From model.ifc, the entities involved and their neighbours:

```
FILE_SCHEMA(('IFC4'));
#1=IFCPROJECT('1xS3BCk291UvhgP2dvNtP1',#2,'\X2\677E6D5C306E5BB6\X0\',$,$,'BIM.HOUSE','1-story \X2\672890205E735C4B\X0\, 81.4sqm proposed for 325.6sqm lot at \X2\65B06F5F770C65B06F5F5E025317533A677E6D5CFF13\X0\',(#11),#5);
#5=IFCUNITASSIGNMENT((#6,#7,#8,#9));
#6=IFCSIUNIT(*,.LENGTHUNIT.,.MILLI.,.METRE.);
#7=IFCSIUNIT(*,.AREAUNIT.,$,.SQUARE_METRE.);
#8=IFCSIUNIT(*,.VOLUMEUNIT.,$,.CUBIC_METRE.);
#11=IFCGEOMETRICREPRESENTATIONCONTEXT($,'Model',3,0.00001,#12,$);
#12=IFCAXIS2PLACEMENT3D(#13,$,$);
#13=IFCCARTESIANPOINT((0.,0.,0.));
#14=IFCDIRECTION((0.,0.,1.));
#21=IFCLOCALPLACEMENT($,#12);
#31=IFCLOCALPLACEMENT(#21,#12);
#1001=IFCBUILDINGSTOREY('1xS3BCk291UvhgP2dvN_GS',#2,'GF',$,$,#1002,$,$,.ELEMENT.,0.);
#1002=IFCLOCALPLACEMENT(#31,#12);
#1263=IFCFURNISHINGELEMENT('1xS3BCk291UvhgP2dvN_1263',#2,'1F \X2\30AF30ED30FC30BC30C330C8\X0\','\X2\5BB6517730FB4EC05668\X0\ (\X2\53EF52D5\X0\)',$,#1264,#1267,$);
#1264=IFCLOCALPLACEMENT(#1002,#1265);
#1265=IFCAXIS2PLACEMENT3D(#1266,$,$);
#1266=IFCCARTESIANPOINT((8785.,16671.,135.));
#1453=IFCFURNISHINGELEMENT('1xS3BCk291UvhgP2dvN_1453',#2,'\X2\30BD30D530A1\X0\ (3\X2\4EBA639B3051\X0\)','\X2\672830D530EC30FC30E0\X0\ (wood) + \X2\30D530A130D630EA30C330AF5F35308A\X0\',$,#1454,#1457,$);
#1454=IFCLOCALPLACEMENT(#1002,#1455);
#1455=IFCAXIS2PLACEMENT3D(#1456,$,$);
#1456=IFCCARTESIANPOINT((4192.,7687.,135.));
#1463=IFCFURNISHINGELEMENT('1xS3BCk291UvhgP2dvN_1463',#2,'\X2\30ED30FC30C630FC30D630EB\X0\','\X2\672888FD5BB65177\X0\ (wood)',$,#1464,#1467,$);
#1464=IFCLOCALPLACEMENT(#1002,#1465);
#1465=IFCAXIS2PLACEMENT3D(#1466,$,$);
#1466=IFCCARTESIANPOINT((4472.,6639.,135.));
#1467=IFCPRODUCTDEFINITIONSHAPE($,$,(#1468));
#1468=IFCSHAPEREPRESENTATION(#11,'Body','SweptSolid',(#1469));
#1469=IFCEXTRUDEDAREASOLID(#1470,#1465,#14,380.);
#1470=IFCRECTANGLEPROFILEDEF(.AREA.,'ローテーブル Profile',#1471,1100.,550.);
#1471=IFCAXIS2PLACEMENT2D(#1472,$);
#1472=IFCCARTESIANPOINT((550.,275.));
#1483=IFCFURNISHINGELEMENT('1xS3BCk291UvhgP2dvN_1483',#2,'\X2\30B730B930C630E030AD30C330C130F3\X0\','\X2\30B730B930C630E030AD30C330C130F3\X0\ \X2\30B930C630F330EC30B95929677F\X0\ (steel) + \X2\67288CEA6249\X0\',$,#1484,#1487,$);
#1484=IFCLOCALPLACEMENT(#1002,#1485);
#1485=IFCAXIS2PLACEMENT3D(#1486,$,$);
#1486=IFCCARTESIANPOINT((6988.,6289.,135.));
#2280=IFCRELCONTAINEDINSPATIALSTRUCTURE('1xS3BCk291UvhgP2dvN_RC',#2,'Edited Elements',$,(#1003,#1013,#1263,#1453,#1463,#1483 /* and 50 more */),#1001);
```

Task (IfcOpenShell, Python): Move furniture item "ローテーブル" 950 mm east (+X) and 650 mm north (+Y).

```python
import ifcopenshell
import ifcopenshell.api.geometry
import ifcopenshell.util.placement
import ifcopenshell.util.unit

model = ifcopenshell.open("model.ifc")
unit_scale = ifcopenshell.util.unit.calculate_unit_scale(model)

item = model.by_guid("1xS3BCk291UvhgP2dvN_1463")
matrix = ifcopenshell.util.placement.get_local_placement(item.ObjectPlacement)
matrix[0, 3] += 0.95 / unit_scale
matrix[1, 3] += 0.65 / unit_scale
ifcopenshell.api.geometry.edit_object_placement(model, product=item, matrix=matrix, is_si=False)

print(ifcopenshell.util.placement.get_local_placement(item.ObjectPlacement).round(3) + 0.0)

model.write("model_edited.ifc")
```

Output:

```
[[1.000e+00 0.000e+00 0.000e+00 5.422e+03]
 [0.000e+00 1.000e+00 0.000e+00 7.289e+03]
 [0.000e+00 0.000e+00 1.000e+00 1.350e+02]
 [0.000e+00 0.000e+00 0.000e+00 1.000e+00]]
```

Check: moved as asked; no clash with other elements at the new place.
